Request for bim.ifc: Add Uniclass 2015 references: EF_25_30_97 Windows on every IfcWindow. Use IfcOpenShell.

First a look at what the model holds.

```python
import ifcopenshell

model = ifcopenshell.open("bim.ifc")
print(model.schema)
print("classifications:", [c.Name for c in model.by_type("IfcClassification")])
for ifc_class in ("IfcDoor", "IfcRoof", "IfcStair", "IfcWall", "IfcWindow"):
    print(ifc_class, len(model.by_type(ifc_class)))
```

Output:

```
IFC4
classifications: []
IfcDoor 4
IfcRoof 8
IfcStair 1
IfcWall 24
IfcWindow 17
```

```python
import ifcopenshell
import ifcopenshell.api.classification

model = ifcopenshell.open("bim.ifc")

system = ifcopenshell.api.classification.add_classification(model, classification="Uniclass 2015")

codes = {
    "IfcWindow": ("EF_25_30_97", "Windows"),
}
for ifc_class, (code, name) in codes.items():
    products = model.by_type(ifc_class)
    ifcopenshell.api.classification.add_reference(
        model, products=products, classification=system, identification=code, name=name
    )
    print(code, len(products))

model.write("bim-out.ifc")
```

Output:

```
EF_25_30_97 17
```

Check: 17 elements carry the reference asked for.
